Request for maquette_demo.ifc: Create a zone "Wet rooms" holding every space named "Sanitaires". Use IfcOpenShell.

First a look at what the model holds.

```python
import ifcopenshell

model = ifcopenshell.open("maquette_demo.ifc")
print(model.schema)
seen = {}
for space in model.by_type("IfcSpace"):
    seen[space.LongName] = seen.get(space.LongName, 0) + 1
for name, count in sorted(seen.items(), key=str):
    print(count, "x", name)
print("zones:", [z.Name for z in model.by_type("IfcZone")][:20])
```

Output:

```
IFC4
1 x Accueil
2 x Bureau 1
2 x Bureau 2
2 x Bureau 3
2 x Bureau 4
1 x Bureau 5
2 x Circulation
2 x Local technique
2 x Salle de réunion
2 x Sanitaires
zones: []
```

```python
import ifcopenshell
import ifcopenshell.api.group
import ifcopenshell.api.root

model = ifcopenshell.open("maquette_demo.ifc")

names = {"Sanitaires"}
spaces = [s for s in model.by_type("IfcSpace") if s.LongName in names]

zone = ifcopenshell.api.root.create_entity(model, ifc_class="IfcZone", name="Wet rooms")
ifcopenshell.api.group.assign_group(model, products=spaces, group=zone)
print(len(spaces), "spaces in", zone.Name)

model.write("maquette_demo-out.ifc")
```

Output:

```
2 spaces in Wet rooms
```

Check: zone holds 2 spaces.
